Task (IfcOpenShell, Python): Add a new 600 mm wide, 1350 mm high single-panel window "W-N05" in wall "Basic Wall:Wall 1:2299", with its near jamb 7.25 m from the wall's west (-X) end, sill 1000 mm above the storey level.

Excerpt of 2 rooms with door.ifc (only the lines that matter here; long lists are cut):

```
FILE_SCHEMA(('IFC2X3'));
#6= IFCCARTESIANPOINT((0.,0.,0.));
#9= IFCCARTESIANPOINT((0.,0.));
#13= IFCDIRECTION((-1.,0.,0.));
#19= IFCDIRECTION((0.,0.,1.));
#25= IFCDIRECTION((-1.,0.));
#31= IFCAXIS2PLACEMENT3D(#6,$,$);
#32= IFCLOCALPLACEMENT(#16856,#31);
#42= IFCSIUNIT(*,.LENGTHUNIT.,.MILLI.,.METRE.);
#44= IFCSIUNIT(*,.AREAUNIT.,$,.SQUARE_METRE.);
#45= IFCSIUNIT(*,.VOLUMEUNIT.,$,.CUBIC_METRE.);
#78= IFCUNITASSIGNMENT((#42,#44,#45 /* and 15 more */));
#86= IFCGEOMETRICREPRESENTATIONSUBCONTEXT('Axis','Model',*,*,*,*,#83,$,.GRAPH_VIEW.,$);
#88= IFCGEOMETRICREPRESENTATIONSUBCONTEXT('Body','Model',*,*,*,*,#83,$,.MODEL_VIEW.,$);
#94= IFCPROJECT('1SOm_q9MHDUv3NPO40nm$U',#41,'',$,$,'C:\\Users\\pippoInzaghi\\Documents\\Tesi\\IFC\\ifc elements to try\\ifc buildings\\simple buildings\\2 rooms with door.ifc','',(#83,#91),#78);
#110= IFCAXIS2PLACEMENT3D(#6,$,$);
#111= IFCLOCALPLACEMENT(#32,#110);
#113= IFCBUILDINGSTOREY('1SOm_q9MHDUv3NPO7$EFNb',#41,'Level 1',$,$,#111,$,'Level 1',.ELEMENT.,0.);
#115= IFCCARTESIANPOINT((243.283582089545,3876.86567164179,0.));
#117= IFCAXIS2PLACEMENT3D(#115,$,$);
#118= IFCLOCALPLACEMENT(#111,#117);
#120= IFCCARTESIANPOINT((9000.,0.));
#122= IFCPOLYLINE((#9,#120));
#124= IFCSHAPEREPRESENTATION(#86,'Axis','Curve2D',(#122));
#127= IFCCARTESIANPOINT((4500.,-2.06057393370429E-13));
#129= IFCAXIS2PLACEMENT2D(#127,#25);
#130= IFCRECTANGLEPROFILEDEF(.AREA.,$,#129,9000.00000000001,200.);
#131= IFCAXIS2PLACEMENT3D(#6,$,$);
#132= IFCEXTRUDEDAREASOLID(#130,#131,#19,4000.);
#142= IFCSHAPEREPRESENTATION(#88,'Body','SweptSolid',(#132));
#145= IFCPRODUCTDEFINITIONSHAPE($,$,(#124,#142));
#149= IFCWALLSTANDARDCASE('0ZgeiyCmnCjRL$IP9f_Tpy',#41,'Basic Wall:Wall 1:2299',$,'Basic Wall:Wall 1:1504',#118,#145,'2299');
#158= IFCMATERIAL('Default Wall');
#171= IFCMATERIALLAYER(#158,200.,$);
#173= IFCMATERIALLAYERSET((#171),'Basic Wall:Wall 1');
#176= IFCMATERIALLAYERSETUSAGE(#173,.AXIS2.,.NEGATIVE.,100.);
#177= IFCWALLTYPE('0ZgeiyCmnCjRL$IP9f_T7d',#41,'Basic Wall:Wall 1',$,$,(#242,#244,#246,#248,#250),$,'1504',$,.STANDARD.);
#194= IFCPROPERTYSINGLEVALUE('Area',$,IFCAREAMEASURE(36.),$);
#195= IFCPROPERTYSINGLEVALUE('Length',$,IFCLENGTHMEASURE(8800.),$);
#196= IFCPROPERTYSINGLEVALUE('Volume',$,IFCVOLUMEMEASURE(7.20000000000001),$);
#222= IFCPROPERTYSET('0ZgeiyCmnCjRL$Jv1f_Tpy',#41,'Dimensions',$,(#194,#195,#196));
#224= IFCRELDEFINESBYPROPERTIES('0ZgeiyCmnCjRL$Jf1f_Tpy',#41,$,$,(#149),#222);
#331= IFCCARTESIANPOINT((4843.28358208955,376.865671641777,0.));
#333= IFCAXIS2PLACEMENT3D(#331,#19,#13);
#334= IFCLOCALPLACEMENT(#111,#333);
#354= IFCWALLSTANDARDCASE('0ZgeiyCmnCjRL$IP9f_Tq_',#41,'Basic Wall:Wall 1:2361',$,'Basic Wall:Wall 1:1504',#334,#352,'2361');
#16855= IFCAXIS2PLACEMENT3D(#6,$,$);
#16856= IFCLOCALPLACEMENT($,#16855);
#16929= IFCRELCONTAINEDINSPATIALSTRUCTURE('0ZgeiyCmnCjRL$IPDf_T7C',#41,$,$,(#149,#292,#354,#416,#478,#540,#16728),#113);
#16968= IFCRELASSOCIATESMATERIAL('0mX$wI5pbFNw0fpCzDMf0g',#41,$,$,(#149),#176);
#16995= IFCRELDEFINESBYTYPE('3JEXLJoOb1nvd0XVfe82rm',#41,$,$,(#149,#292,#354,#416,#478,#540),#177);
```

```python
import numpy as np
import ifcopenshell
import ifcopenshell.api.feature
import ifcopenshell.api.geometry
import ifcopenshell.api.pset
import ifcopenshell.api.root
import ifcopenshell.api.spatial
import ifcopenshell.api.type
import ifcopenshell.geom
import ifcopenshell.util.element
import ifcopenshell.util.placement
import ifcopenshell.util.representation
import ifcopenshell.util.shape
import ifcopenshell.util.unit

model = ifcopenshell.open("2 rooms with door.ifc")
unit_scale = ifcopenshell.util.unit.calculate_unit_scale(model)
area_scale = ifcopenshell.util.unit.calculate_unit_scale(model, "AREAUNIT")
volume_scale = ifcopenshell.util.unit.calculate_unit_scale(model, "VOLUMEUNIT")
settings = ifcopenshell.geom.settings()


def volume(element):
    """Net volume in cubic metres, openings subtracted."""
    shape = ifcopenshell.geom.create_shape(settings, element)
    return ifcopenshell.util.shape.get_volume(shape.geometry)


wall = model.by_id(149)
storey = ifcopenshell.util.element.get_container(wall, ifc_class="IfcBuildingStorey")
context = ifcopenshell.util.representation.get_context(model, "Model", "Body", "MODEL_VIEW")
before = volume(wall)

width, height, from_end, sill = 0.6, 1.35, 7.25, 1  # metres

# The wall runs along its own X axis, and the end named is its -X end.
wall_shape = ifcopenshell.geom.create_shape(settings, wall)
x, y, z = ifcopenshell.util.shape.get_vertices(wall_shape.geometry).T
start = x.min() + from_end
face, thickness = float(y.min()), float(y.max() - y.min())
wall_matrix = ifcopenshell.util.placement.get_local_placement(wall.ObjectPlacement)
level = ifcopenshell.util.placement.get_local_placement(storey.ObjectPlacement)[2, 3]


def in_wall(x, y):
    """Placement at x, y metres in the wall's axes, at sill height."""
    matrix = wall_matrix.copy()
    matrix[:, 3] = wall_matrix @ np.array([x / unit_scale, y / unit_scale, 0.0, 1.0])
    matrix[2, 3] = level + sill / unit_scale
    return matrix


# Opening: a box that overshoots both wall faces by 50 mm.
opening = ifcopenshell.api.root.create_entity(model, ifc_class="IfcOpeningElement")
box = ifcopenshell.api.geometry.add_wall_representation(
    model, context=context, length=width, height=height, thickness=thickness + 0.1
)
ifcopenshell.api.geometry.assign_representation(model, product=opening, representation=box)
ifcopenshell.api.geometry.edit_object_placement(model, product=opening, matrix=in_wall(start, face - 0.05), is_si=False)
ifcopenshell.api.feature.add_feature(model, feature=opening, element=wall)

window = ifcopenshell.api.root.create_entity(model, ifc_class="IfcWindow", name="W-N05")
window.OverallWidth, window.OverallHeight = width / unit_scale, height / unit_scale
body = ifcopenshell.api.geometry.add_window_representation(
    model,
    context=context,
    overall_width=window.OverallWidth,
    overall_height=window.OverallHeight,
    partition_type="SINGLE_PANEL",
)
ifcopenshell.api.geometry.assign_representation(model, product=window, representation=body)
ifcopenshell.api.spatial.assign_container(model, products=[window], relating_structure=storey)
fills = ifcopenshell.api.feature.add_filling(model, opening=opening, element=window)
fills.OwnerHistory = window.OwnerHistory  # required in IFC2X3

# IFC2X3 keeps the operation on the window style.
style = ifcopenshell.api.root.create_entity(model, ifc_class="IfcWindowStyle", name="W-N05")
style.OperationType, style.ConstructionType = "SINGLE_PANEL", "NOTDEFINED"
style.ParameterTakesPrecedence = style.Sizeable = False
ifcopenshell.api.type.assign_type(model, related_objects=[window], relating_type=style)

# Centre the window in the wall's thickness.
ifcopenshell.api.geometry.edit_object_placement(model, product=window, matrix=in_wall(start, face), is_si=False)
window_shape = ifcopenshell.geom.create_shape(settings, window)
depth = ifcopenshell.util.shape.get_vertices(window_shape.geometry)[:, 1]
offset = face + thickness / 2 - (depth.min() + depth.max()) / 2
ifcopenshell.api.geometry.edit_object_placement(model, product=window, matrix=in_wall(start, offset), is_si=False)

after = volume(wall)

# Update the wall's stored quantities.
pset = model.by_id(ifcopenshell.util.element.get_pset(wall, "Dimensions", should_inherit=False)["id"])
ifcopenshell.api.pset.edit_pset(model, pset=pset, properties={
    "Area": model.create_entity("IfcAreaMeasure", after / thickness / area_scale),
    "Volume": model.create_entity("IfcVolumeMeasure", after / volume_scale),
})

print(f"wall volume {before:.3f} -> {after:.3f} m3")

model.write("2 rooms with door_rev.ifc")
```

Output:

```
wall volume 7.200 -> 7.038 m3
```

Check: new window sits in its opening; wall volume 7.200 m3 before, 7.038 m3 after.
